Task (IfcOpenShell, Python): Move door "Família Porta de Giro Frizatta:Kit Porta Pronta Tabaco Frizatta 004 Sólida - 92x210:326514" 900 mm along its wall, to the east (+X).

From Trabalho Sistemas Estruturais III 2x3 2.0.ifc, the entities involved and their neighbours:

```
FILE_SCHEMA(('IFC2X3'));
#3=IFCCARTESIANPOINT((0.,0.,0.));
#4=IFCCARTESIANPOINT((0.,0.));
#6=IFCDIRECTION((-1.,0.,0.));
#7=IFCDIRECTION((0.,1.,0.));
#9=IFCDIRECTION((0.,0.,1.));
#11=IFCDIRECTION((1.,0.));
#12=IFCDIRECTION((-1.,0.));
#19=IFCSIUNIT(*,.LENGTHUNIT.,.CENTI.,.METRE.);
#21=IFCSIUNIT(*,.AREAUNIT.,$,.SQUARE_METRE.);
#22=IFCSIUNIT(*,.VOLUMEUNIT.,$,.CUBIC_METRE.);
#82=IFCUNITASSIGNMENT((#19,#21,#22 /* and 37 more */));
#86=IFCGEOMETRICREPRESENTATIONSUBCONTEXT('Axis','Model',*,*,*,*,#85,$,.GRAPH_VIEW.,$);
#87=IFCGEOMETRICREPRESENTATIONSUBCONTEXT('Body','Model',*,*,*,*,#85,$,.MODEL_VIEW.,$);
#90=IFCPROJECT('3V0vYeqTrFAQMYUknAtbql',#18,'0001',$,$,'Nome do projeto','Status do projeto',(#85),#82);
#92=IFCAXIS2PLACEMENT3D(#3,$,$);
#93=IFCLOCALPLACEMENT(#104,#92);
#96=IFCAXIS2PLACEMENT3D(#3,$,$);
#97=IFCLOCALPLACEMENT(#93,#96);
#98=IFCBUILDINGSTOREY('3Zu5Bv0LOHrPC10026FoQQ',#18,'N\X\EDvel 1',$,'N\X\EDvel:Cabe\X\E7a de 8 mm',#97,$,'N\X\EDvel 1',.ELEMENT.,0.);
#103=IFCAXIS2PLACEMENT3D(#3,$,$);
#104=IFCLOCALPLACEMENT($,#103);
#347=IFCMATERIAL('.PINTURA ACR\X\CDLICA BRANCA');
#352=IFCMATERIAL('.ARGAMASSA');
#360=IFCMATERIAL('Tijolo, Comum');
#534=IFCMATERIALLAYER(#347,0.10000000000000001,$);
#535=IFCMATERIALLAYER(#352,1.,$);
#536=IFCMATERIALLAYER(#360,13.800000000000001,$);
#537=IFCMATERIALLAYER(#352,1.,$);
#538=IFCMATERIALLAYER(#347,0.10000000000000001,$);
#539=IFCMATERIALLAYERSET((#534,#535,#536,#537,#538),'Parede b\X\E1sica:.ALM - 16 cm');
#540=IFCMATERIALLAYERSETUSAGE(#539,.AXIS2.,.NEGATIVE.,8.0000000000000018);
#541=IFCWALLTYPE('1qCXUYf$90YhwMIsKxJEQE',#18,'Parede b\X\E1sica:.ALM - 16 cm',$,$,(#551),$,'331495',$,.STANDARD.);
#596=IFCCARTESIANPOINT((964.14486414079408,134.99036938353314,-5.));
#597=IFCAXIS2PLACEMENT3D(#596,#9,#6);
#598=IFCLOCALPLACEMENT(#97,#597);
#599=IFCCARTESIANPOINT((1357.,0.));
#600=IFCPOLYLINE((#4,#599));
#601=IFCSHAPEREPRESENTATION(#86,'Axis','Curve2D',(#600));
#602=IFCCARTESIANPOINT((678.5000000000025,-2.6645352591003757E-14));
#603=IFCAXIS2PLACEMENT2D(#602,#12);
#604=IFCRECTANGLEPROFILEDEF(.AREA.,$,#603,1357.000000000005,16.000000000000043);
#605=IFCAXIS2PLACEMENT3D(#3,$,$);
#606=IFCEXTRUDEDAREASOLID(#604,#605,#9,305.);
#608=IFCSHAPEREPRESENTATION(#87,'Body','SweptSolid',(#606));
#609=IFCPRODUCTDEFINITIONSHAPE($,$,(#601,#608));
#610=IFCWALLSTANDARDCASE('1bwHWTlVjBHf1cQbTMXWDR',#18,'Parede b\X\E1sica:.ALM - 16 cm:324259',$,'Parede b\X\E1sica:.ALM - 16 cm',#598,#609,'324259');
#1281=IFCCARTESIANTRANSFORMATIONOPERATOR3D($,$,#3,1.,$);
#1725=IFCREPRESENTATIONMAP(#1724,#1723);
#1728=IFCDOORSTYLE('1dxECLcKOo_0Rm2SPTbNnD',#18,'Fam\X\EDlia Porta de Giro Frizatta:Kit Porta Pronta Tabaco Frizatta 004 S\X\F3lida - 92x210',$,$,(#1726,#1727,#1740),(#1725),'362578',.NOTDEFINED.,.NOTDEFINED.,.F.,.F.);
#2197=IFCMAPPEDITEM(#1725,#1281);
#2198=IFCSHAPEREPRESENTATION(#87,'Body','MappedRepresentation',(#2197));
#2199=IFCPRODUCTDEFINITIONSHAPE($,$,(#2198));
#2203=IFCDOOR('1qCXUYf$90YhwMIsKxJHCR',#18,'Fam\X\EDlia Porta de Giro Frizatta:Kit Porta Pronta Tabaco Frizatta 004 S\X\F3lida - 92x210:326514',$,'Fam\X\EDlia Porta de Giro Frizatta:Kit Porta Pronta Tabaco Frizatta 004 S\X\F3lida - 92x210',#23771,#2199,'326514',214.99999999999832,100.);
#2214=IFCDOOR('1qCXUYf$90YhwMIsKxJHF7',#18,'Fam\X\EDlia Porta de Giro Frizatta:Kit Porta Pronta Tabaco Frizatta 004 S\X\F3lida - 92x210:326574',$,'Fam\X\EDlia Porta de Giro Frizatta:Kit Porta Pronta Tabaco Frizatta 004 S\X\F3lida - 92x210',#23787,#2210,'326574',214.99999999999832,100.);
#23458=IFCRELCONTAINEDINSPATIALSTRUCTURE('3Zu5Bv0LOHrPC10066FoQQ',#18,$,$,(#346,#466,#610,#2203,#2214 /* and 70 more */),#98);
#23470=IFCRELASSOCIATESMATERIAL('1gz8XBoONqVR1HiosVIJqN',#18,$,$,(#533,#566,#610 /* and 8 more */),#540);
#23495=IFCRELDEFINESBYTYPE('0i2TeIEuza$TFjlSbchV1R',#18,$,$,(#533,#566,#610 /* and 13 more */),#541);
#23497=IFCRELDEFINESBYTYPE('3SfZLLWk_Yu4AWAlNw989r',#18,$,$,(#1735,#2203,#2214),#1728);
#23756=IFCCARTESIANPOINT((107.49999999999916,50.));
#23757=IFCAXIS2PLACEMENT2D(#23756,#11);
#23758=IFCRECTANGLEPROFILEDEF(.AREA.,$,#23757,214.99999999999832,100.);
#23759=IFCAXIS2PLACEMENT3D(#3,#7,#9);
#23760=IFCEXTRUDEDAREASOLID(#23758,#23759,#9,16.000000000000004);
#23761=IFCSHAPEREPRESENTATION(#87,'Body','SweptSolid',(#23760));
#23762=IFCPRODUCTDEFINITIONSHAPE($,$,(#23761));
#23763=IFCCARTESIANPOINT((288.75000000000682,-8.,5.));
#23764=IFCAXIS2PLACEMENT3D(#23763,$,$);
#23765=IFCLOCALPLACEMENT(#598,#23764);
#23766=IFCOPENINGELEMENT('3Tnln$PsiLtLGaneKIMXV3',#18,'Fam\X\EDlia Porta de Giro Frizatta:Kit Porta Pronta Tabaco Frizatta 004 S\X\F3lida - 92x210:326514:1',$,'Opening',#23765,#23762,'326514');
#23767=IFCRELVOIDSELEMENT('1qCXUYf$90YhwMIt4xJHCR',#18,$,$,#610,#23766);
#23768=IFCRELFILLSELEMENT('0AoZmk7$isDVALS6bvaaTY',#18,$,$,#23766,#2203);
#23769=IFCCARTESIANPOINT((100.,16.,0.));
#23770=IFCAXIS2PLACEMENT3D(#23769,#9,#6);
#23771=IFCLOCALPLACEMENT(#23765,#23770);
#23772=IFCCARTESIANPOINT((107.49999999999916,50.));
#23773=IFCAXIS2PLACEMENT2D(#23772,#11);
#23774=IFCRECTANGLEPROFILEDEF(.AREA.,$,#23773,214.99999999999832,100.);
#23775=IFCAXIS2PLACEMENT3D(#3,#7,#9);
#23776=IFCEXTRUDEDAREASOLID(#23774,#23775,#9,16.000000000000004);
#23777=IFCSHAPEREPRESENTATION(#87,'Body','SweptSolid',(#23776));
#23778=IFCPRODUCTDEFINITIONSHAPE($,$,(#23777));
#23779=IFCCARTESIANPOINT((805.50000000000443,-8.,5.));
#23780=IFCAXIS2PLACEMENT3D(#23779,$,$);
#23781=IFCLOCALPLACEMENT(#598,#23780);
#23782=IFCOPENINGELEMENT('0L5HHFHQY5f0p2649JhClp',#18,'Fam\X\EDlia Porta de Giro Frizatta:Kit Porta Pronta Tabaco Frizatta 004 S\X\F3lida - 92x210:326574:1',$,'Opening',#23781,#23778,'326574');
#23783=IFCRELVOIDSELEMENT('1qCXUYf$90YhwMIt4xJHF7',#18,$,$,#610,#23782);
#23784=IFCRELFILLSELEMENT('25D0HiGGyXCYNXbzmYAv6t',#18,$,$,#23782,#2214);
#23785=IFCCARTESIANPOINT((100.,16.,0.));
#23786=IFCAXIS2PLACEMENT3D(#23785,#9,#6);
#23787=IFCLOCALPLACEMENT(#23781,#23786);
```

```python
import ifcopenshell
import ifcopenshell.api.geometry
import ifcopenshell.util.placement
import ifcopenshell.util.unit

model = ifcopenshell.open("Trabalho Sistemas Estruturais III 2x3 2.0.ifc")
unit_scale = ifcopenshell.util.unit.calculate_unit_scale(model)

door = model.by_id(2203)
opening = door.FillsVoids[0].RelatingOpeningElement
wall = opening.VoidsElements[0].RelatingBuildingElement

wall_matrix = ifcopenshell.util.placement.get_local_placement(wall.ObjectPlacement)
shift = wall_matrix[:3, 0] * -0.9 / unit_scale
before = ifcopenshell.util.placement.get_local_placement(door.ObjectPlacement)[:3, 3].copy()

# The door is placed relative to its opening, so it follows when the opening moves.
matrix = ifcopenshell.util.placement.get_local_placement(opening.ObjectPlacement)
matrix[:3, 3] += shift
ifcopenshell.api.geometry.edit_object_placement(
    model, product=opening, matrix=matrix, is_si=False, should_transform_children=True
)

after = ifcopenshell.util.placement.get_local_placement(door.ObjectPlacement)[:3, 3]
print("door moved by", (after - before).round(3) + 0.0)

model.write("Trabalho Sistemas Estruturais III 2x3 2.0_updated.ifc")
```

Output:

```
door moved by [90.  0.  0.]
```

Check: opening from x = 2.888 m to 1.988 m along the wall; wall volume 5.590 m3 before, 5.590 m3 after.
